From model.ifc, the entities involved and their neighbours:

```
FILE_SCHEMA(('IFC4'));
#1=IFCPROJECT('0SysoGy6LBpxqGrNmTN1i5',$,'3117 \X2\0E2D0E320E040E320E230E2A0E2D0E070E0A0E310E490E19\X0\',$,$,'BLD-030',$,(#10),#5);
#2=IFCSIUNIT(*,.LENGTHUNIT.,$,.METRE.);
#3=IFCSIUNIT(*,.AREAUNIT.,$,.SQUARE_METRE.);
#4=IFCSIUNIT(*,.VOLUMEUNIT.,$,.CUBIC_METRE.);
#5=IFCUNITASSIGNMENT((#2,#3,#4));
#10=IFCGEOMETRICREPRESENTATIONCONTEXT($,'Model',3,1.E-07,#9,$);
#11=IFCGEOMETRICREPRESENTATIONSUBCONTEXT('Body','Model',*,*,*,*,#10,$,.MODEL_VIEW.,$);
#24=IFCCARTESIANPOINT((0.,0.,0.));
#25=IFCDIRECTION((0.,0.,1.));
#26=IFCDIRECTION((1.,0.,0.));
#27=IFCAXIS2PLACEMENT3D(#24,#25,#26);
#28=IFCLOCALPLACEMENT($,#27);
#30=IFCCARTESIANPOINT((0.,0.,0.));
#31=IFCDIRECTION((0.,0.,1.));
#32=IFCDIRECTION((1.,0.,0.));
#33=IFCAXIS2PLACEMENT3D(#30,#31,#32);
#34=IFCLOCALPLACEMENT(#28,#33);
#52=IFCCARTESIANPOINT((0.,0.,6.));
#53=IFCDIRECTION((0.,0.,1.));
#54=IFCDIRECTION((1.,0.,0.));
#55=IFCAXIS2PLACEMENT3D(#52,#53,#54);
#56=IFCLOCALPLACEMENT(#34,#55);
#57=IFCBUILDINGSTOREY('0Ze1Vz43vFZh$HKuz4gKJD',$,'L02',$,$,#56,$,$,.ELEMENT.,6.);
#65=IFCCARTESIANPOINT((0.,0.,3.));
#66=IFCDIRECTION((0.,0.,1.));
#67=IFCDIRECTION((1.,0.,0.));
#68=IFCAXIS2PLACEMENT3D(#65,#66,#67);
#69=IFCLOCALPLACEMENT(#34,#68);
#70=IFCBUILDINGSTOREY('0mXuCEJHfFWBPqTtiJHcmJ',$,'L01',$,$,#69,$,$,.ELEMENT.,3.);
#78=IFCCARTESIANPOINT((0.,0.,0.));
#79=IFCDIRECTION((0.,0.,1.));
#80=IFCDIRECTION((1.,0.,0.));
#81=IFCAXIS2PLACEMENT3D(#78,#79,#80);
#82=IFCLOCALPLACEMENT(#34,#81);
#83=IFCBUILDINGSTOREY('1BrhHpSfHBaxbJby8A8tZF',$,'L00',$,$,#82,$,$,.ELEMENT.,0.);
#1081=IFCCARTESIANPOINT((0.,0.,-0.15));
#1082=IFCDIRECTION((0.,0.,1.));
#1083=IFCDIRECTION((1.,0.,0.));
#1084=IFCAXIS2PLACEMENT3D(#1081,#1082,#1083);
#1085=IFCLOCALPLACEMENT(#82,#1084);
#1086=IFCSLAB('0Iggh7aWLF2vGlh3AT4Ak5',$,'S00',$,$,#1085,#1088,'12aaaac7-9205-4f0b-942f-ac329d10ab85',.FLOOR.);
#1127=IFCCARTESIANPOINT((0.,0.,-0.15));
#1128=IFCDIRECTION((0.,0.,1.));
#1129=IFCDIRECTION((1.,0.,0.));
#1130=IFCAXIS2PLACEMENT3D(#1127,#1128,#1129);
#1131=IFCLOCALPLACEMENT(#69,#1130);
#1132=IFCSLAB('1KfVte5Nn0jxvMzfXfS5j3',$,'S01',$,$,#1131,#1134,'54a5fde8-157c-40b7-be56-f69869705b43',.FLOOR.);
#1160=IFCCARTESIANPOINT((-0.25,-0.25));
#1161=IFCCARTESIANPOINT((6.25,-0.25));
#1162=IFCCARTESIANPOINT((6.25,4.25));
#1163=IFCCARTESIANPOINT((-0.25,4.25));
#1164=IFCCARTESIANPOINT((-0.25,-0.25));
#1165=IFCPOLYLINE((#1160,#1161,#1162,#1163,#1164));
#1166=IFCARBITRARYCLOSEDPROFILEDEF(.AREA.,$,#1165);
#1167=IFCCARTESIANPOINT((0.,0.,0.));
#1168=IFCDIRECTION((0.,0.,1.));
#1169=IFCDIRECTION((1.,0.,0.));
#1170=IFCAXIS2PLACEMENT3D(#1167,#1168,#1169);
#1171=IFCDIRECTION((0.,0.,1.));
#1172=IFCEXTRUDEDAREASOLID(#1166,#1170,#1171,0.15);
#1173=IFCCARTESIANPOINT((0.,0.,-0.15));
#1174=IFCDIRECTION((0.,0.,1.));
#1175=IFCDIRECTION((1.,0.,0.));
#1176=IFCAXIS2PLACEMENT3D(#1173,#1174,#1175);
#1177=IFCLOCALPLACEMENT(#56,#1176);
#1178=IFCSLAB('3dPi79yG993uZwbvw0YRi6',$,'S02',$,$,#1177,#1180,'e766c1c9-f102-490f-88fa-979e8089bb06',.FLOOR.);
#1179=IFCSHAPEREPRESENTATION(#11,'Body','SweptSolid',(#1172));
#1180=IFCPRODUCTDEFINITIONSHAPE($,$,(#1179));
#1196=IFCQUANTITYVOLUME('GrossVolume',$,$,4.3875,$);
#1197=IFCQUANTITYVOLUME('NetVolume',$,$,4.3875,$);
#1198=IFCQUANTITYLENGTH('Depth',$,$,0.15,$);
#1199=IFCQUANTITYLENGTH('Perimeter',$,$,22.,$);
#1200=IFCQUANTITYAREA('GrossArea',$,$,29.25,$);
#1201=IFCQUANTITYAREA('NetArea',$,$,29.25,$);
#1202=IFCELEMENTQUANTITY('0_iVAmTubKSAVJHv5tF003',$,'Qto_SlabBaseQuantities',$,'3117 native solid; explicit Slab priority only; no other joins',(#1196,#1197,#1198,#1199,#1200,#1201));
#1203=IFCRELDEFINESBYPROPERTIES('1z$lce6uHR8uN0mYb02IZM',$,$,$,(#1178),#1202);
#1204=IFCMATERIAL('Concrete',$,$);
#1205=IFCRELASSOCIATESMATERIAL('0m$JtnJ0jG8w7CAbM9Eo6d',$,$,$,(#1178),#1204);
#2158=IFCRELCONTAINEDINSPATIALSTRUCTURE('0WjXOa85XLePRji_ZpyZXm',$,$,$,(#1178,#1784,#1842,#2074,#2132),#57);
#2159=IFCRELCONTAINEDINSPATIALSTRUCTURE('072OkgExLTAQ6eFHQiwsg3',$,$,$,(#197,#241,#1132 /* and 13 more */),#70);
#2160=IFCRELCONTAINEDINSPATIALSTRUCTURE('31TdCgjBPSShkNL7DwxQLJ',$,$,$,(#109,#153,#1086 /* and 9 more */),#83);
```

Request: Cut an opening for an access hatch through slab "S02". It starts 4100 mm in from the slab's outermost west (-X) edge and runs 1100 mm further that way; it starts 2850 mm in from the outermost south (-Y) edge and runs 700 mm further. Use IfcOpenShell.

```python
import numpy as np
import ifcopenshell
import ifcopenshell.api.feature
import ifcopenshell.api.geometry
import ifcopenshell.api.pset
import ifcopenshell.api.root
import ifcopenshell.geom
import ifcopenshell.util.element
import ifcopenshell.util.placement
import ifcopenshell.util.representation
import ifcopenshell.util.shape
import ifcopenshell.util.unit

model = ifcopenshell.open("model.ifc")
unit_scale = ifcopenshell.util.unit.calculate_unit_scale(model)
area_scale = ifcopenshell.util.unit.calculate_unit_scale(model, "AREAUNIT")
volume_scale = ifcopenshell.util.unit.calculate_unit_scale(model, "VOLUMEUNIT")
settings = ifcopenshell.geom.settings()


def volume(element):
    """Net volume in cubic metres, openings subtracted."""
    shape = ifcopenshell.geom.create_shape(settings, element)
    return ifcopenshell.util.shape.get_volume(shape.geometry)


slab = model.by_guid("3dPi79yG993uZwbvw0YRi6")
before = volume(slab)

# Extent in the slab's own axes, in metres. The edges named are its -X and -Y sides.
slab_shape = ifcopenshell.geom.create_shape(settings, slab)
vertices = ifcopenshell.util.shape.get_vertices(slab_shape.geometry)
x_min, y_min, bottom = vertices.min(axis=0)
top = vertices[:, 2].max()

opening = ifcopenshell.api.root.create_entity(model, ifc_class="IfcOpeningElement", name="Access hatch opening", predefined_type="OPENING")
context = ifcopenshell.util.representation.get_context(model, "Model", "Body", "MODEL_VIEW")
width, depth = 1.1, 0.7
outline = [(0.0, 0.0), (width, 0.0), (width, depth), (0.0, depth), (0.0, 0.0)]
# Overshoot both faces by 50 mm so the cut is clean.
shape = ifcopenshell.api.geometry.add_slab_representation(
    model, context=context, depth=top - bottom + 0.1, polyline=outline
)
ifcopenshell.api.geometry.assign_representation(model, product=opening, representation=shape)

matrix = ifcopenshell.util.placement.get_local_placement(slab.ObjectPlacement)
matrix[:, 3] = matrix @ np.append(np.array([x_min + 4.1, y_min + 2.85, bottom - 0.05]) / unit_scale, 1.0)
ifcopenshell.api.geometry.edit_object_placement(model, product=opening, matrix=matrix, is_si=False)
ifcopenshell.api.feature.add_feature(model, feature=opening, element=slab)

after = volume(slab)

# Update the slab's stored quantities.
qto = model.by_id(ifcopenshell.util.element.get_pset(slab, "Qto_SlabBaseQuantities", should_inherit=False)["id"])
ifcopenshell.api.pset.edit_qto(model, qto=qto, properties={
    "NetVolume": after / volume_scale,
    "NetArea": after / (top - bottom) / area_scale,
})

print(f"slab volume {before:.3f} -> {after:.3f} m3")

model.write("model-out.ifc")
```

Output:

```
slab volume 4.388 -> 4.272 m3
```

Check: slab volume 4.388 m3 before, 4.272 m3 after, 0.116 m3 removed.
